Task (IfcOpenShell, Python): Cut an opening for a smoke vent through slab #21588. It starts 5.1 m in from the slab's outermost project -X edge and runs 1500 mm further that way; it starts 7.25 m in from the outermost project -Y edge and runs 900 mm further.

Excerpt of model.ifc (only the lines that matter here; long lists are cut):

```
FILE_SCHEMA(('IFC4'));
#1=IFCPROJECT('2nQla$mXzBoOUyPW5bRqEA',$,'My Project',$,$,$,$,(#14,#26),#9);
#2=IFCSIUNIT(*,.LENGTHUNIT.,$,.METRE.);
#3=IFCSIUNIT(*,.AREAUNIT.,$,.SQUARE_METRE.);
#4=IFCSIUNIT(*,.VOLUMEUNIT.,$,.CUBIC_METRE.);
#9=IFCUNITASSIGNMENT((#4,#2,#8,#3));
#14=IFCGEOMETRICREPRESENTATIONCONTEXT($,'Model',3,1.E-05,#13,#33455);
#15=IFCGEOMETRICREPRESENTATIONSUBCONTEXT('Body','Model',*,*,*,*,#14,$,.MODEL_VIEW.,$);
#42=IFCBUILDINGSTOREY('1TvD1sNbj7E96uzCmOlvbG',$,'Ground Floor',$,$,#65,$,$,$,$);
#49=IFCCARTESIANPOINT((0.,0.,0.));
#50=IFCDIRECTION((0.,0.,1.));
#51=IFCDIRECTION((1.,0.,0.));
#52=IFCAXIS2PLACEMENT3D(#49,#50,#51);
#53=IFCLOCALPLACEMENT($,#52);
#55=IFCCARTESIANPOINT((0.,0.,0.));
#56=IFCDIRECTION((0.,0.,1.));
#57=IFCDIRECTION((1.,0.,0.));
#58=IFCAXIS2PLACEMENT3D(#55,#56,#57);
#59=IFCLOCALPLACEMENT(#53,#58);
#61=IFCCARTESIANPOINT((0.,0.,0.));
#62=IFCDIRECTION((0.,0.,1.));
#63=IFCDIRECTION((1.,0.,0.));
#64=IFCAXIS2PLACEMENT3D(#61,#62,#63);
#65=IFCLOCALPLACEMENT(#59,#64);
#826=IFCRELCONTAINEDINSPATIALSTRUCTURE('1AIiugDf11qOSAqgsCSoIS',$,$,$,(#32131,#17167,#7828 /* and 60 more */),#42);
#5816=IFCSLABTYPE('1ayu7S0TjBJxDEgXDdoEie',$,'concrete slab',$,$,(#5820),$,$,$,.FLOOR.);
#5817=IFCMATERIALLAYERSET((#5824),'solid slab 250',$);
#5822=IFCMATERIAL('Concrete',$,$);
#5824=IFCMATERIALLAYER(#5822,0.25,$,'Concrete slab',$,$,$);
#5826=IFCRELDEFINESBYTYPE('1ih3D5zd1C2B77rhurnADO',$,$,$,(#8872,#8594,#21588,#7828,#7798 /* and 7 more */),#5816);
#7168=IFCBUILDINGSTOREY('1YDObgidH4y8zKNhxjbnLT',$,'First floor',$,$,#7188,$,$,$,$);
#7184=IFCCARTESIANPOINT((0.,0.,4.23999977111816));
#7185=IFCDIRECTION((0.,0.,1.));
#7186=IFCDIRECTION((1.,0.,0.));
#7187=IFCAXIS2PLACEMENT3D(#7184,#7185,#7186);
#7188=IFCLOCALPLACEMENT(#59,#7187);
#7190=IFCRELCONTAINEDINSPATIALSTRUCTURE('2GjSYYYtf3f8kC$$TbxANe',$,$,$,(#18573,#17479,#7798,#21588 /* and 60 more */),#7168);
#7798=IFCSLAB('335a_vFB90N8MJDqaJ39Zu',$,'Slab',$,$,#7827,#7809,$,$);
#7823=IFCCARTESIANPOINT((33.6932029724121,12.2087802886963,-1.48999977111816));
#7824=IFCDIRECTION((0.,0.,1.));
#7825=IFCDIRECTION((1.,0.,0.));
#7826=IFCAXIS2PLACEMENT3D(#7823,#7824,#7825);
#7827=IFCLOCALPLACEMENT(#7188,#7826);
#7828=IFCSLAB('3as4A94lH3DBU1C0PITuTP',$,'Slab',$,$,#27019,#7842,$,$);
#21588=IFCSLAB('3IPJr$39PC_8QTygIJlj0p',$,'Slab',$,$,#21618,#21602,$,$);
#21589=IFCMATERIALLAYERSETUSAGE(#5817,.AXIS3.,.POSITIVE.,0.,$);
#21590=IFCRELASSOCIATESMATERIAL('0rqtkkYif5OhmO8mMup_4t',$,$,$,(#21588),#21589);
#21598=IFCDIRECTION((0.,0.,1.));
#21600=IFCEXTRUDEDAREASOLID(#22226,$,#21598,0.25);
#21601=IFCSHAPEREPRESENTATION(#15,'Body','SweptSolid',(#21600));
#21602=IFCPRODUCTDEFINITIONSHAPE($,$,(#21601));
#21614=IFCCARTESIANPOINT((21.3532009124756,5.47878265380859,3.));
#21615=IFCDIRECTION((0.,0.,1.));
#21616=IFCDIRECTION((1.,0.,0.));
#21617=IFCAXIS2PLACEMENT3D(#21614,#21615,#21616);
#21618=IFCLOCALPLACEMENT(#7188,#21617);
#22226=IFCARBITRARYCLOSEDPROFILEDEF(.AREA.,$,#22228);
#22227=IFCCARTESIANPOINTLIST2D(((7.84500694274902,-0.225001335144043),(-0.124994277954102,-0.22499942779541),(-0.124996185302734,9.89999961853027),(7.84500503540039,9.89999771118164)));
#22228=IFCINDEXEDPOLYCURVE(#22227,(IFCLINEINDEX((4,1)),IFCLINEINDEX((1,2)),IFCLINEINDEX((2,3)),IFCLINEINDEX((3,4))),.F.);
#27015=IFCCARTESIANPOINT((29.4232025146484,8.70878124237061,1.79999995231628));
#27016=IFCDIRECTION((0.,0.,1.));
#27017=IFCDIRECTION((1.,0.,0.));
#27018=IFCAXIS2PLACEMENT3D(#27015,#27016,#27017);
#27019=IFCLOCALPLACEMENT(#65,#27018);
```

```python
import numpy as np
import ifcopenshell
import ifcopenshell.api.feature
import ifcopenshell.api.geometry
import ifcopenshell.api.root
import ifcopenshell.geom
import ifcopenshell.util.placement
import ifcopenshell.util.representation
import ifcopenshell.util.shape
import ifcopenshell.util.unit

model = ifcopenshell.open("model.ifc")
unit_scale = ifcopenshell.util.unit.calculate_unit_scale(model)
settings = ifcopenshell.geom.settings()


def volume(element):
    """Net volume in cubic metres, openings subtracted."""
    shape = ifcopenshell.geom.create_shape(settings, element)
    return ifcopenshell.util.shape.get_volume(shape.geometry)


slab = model.by_guid("3IPJr$39PC_8QTygIJlj0p")
before = volume(slab)

# Extent in the slab's own axes, in metres. The edges named are its -X and -Y sides.
slab_shape = ifcopenshell.geom.create_shape(settings, slab)
vertices = ifcopenshell.util.shape.get_vertices(slab_shape.geometry)
x_min, y_min, bottom = vertices.min(axis=0)
top = vertices[:, 2].max()

opening = ifcopenshell.api.root.create_entity(model, ifc_class="IfcOpeningElement", name="Smoke vent opening", predefined_type="OPENING")
context = ifcopenshell.util.representation.get_context(model, "Model", "Body", "MODEL_VIEW")
width, depth = 1.5, 0.9
outline = [(0.0, 0.0), (width, 0.0), (width, depth), (0.0, depth), (0.0, 0.0)]
# Overshoot both faces by 50 mm so the cut is clean.
shape = ifcopenshell.api.geometry.add_slab_representation(
    model, context=context, depth=top - bottom + 0.1, polyline=outline
)
ifcopenshell.api.geometry.assign_representation(model, product=opening, representation=shape)

matrix = ifcopenshell.util.placement.get_local_placement(slab.ObjectPlacement)
matrix[:, 3] = matrix @ np.append(np.array([x_min + 5.1, y_min + 7.25, bottom - 0.05]) / unit_scale, 1.0)
ifcopenshell.api.geometry.edit_object_placement(model, product=opening, matrix=matrix, is_si=False)
ifcopenshell.api.feature.add_feature(model, feature=opening, element=slab)

after = volume(slab)

print(f"slab volume {before:.3f} -> {after:.3f} m3")

model.write("model_edited.ifc")
```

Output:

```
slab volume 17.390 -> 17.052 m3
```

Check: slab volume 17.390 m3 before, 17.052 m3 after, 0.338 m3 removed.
